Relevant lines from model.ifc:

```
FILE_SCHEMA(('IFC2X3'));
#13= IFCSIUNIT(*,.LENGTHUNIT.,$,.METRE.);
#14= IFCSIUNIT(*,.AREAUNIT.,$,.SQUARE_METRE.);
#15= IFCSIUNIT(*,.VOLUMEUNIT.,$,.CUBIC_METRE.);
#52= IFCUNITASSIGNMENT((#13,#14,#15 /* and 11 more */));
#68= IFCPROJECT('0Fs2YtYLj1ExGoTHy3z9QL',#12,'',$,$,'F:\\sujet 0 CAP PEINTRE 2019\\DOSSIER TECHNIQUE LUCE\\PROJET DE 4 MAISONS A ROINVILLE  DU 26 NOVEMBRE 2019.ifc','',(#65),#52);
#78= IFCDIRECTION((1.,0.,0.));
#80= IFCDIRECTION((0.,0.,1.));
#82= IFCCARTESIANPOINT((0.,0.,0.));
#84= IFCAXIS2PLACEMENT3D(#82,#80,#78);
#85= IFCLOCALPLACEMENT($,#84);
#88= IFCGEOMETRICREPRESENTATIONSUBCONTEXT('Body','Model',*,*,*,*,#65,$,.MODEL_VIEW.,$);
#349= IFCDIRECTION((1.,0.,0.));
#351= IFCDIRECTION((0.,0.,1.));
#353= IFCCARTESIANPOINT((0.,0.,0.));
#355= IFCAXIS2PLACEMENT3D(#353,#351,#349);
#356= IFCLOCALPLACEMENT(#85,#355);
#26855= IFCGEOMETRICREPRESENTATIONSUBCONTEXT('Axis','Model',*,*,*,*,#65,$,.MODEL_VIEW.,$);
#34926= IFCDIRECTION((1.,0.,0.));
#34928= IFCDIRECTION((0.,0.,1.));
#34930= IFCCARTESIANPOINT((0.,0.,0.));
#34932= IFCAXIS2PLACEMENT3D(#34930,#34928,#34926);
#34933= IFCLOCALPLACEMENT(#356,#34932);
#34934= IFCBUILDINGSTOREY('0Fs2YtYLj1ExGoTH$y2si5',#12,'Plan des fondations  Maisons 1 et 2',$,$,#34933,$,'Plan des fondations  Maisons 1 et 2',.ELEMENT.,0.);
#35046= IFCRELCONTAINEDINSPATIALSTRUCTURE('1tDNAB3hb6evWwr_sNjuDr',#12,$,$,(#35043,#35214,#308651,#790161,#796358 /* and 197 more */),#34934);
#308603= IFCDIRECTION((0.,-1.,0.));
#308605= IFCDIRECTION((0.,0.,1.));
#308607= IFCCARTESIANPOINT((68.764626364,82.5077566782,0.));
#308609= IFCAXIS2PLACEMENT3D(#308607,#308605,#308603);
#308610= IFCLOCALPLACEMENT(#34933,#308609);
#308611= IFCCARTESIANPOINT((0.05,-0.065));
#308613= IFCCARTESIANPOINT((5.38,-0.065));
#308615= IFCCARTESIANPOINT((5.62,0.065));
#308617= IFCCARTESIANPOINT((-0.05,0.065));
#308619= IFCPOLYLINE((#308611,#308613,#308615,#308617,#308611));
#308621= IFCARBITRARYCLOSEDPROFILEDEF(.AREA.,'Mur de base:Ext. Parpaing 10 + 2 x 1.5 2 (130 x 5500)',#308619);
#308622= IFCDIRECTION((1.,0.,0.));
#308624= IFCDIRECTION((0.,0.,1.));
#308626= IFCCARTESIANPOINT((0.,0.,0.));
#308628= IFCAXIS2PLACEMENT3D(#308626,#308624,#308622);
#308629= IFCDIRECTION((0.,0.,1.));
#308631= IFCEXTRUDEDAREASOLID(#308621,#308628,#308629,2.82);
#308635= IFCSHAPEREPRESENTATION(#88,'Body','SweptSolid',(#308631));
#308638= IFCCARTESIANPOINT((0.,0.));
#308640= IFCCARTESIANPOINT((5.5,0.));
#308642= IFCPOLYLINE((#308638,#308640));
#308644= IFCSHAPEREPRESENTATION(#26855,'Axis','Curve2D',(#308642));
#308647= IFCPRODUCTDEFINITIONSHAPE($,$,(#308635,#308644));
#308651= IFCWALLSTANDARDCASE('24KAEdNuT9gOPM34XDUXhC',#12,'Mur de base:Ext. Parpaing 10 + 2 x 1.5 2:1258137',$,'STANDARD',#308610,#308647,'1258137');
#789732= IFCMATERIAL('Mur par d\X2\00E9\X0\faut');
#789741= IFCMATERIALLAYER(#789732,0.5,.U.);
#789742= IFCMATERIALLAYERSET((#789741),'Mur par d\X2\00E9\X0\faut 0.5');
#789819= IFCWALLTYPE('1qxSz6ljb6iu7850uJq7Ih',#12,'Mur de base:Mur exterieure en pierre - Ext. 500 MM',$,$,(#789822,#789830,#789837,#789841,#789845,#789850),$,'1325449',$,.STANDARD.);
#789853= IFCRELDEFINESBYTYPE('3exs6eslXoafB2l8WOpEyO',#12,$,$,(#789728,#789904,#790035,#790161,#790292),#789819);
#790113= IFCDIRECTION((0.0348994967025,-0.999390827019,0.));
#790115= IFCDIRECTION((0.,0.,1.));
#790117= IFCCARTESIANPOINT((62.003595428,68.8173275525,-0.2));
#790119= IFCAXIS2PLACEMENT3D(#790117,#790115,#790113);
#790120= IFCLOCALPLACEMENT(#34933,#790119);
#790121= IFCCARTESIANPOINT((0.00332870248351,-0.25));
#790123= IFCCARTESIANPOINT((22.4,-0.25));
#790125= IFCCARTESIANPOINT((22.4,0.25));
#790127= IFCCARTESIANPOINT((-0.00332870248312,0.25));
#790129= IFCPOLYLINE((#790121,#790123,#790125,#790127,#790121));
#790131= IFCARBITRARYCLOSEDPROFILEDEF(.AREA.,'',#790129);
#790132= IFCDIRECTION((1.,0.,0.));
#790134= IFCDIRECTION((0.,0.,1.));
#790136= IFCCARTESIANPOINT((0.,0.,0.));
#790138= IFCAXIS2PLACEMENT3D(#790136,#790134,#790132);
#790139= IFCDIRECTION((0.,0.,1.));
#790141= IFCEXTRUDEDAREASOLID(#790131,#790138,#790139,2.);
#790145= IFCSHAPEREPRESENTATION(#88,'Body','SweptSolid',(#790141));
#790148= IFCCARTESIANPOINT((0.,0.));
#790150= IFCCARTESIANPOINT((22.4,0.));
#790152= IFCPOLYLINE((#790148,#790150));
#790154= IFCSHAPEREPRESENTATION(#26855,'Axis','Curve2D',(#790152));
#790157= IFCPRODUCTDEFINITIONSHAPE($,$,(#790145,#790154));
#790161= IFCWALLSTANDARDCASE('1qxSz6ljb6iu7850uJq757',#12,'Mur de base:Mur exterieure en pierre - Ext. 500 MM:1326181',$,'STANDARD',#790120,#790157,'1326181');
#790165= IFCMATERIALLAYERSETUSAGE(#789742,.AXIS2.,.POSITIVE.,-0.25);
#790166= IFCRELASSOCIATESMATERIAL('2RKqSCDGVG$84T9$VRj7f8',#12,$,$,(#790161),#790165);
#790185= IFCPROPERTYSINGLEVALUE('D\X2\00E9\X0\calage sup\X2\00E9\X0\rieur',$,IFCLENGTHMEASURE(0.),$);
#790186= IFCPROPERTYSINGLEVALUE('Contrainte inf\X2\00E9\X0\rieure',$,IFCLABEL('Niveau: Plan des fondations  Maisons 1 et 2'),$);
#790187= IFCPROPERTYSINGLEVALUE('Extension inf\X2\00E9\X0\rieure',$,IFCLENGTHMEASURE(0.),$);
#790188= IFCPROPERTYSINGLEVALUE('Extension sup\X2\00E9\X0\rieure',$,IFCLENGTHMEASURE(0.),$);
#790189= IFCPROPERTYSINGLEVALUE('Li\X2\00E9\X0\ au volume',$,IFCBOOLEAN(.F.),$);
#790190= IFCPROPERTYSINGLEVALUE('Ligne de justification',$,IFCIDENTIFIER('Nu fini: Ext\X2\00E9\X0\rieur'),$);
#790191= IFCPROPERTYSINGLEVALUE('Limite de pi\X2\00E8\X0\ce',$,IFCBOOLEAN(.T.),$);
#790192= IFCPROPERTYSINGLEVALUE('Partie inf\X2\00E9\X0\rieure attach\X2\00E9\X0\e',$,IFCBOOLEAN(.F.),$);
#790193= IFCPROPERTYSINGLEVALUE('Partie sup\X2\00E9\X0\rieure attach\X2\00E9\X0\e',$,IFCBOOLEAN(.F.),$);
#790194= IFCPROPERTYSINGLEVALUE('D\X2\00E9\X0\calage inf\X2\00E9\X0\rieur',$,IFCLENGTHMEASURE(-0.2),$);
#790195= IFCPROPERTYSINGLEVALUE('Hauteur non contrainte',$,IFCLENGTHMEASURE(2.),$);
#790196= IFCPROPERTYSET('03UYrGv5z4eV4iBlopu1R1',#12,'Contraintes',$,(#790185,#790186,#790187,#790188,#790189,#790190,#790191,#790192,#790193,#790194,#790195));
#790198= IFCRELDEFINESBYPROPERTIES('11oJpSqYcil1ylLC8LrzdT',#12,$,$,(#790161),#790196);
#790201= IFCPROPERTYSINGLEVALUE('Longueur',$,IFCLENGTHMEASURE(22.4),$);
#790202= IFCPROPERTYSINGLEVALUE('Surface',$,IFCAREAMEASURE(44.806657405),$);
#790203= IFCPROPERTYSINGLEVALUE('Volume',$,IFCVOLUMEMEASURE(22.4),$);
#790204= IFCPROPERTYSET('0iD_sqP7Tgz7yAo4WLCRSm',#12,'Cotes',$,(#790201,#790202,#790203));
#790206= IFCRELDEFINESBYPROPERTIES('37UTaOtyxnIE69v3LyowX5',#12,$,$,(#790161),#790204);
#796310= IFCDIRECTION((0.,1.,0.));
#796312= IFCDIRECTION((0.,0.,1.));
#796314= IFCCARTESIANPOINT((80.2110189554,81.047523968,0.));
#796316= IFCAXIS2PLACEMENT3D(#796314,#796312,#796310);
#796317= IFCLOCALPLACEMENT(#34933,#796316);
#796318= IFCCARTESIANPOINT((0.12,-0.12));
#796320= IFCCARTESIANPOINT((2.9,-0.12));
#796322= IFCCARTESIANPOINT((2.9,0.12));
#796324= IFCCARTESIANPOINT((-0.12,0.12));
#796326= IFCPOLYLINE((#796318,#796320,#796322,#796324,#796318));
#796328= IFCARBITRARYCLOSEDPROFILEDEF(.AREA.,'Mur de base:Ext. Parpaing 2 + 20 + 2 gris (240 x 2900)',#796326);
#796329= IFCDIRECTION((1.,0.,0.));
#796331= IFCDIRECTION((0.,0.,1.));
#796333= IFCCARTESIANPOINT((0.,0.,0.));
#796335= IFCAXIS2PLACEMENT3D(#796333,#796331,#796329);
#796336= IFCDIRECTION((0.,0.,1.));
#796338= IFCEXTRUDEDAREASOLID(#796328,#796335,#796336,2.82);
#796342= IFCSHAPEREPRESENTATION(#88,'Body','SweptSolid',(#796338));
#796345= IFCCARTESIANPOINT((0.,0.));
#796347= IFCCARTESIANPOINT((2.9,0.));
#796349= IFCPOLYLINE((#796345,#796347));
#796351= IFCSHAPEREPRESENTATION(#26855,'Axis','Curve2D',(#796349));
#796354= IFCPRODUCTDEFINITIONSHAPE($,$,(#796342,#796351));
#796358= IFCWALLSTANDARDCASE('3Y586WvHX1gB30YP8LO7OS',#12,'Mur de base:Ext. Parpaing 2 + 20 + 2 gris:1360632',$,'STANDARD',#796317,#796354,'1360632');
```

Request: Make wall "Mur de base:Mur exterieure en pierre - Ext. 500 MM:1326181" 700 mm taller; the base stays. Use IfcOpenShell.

```python
import ifcopenshell
import ifcopenshell.api.pset
import ifcopenshell.geom
import ifcopenshell.util.element
import ifcopenshell.util.representation
import ifcopenshell.util.shape
import ifcopenshell.util.unit

model = ifcopenshell.open("model.ifc")
unit_scale = ifcopenshell.util.unit.calculate_unit_scale(model)
area_scale = ifcopenshell.util.unit.calculate_unit_scale(model, "AREAUNIT")
volume_scale = ifcopenshell.util.unit.calculate_unit_scale(model, "VOLUMEUNIT")
settings = ifcopenshell.geom.settings()


def volume(element):
    """Net volume in cubic metres, openings subtracted."""
    shape = ifcopenshell.geom.create_shape(settings, element)
    return ifcopenshell.util.shape.get_volume(shape.geometry)


wall = model.by_guid("1qxSz6ljb6iu7850uJq757")
before = volume(wall)

body = ifcopenshell.util.representation.get_representation(wall, "Model", "Body")
solid = body.Items[0]
old_height = solid.Depth
solid.Depth += 0.7 / unit_scale
after = volume(wall)
thickness = 0.5  # wall thickness in metres

# Update the stored height, areas and volumes.
pset = model.by_id(ifcopenshell.util.element.get_pset(wall, "Contraintes", should_inherit=False)["id"])
ifcopenshell.api.pset.edit_pset(model, pset=pset, properties={
    "Hauteur non contrainte": model.create_entity("IfcLengthMeasure", solid.Depth),
})
pset = model.by_id(ifcopenshell.util.element.get_pset(wall, "Cotes", should_inherit=False)["id"])
ifcopenshell.api.pset.edit_pset(model, pset=pset, properties={
    "Surface": model.create_entity("IfcAreaMeasure", after / thickness / area_scale),
    "Volume": model.create_entity("IfcVolumeMeasure", after / volume_scale),
})

print(f"height {old_height:g} -> {solid.Depth:g}, volume {before:.3f} -> {after:.3f} m3")

model.write("model_updated.ifc")
```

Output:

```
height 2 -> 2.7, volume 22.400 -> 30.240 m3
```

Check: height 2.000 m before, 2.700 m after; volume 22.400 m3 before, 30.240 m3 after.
